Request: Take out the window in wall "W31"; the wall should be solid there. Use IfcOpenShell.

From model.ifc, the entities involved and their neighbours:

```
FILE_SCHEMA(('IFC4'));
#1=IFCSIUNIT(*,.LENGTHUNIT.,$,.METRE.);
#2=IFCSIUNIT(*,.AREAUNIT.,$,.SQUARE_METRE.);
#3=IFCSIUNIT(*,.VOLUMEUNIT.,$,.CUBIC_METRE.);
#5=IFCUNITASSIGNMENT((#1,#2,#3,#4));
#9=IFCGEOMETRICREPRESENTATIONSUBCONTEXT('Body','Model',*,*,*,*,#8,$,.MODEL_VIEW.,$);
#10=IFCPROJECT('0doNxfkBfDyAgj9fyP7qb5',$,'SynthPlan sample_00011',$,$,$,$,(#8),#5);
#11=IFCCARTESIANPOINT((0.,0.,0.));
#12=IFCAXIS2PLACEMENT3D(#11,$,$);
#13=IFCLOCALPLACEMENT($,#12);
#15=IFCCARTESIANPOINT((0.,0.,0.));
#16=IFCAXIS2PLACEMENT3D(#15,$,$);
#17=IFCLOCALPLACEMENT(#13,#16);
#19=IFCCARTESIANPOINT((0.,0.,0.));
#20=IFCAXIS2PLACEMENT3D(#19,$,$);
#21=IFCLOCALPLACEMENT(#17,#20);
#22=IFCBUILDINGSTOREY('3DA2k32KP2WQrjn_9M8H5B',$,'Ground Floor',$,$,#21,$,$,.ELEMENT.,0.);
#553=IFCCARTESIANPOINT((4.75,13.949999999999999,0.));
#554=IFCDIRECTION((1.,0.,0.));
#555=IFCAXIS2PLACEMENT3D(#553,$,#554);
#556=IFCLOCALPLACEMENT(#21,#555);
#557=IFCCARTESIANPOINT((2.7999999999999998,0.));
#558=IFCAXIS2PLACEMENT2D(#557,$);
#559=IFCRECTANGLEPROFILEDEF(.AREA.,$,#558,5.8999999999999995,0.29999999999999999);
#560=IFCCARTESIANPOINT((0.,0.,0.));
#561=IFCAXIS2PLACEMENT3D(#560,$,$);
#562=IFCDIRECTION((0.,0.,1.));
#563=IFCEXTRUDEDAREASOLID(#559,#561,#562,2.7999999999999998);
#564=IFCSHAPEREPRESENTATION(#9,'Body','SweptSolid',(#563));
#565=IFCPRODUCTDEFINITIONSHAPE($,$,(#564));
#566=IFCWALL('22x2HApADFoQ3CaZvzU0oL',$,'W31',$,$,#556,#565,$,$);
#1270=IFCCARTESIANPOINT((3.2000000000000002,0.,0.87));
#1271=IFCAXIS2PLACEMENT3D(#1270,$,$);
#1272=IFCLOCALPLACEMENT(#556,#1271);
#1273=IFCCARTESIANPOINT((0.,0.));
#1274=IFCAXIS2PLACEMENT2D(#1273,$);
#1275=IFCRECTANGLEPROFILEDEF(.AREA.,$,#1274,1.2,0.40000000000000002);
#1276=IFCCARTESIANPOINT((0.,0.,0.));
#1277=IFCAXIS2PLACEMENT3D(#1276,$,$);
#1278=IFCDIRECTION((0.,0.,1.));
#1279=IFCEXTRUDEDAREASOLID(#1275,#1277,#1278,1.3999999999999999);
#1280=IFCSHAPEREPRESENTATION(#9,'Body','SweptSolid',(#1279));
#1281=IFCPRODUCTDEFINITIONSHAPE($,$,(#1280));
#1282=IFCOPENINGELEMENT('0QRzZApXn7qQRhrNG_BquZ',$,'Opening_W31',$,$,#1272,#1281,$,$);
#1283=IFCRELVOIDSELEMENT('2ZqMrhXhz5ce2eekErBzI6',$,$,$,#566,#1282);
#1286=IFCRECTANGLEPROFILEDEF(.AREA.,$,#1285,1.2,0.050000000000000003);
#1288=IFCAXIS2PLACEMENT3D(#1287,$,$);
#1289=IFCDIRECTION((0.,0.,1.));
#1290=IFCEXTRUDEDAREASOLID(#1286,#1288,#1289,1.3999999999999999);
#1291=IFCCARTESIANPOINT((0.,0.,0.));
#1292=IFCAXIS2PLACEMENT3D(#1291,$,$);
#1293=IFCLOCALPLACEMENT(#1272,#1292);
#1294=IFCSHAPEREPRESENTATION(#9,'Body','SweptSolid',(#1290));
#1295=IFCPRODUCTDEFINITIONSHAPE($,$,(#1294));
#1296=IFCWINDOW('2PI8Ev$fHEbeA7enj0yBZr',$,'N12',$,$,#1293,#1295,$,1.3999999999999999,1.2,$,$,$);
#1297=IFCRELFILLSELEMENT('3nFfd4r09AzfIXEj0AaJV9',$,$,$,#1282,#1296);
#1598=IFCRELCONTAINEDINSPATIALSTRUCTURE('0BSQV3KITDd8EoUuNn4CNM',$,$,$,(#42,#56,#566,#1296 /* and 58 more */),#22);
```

```python
import ifcopenshell
import ifcopenshell.api.feature
import ifcopenshell.api.root
import ifcopenshell.geom
import ifcopenshell.util.shape

model = ifcopenshell.open("model.ifc")
settings = ifcopenshell.geom.settings()


def volume(element):
    """Net volume in cubic metres, openings subtracted."""
    shape = ifcopenshell.geom.create_shape(settings, element)
    return ifcopenshell.util.shape.get_volume(shape.geometry)


window = model.by_guid("2PI8Ev$fHEbeA7enj0yBZr")
opening = window.FillsVoids[0].RelatingOpeningElement
wall = opening.VoidsElements[0].RelatingBuildingElement
before = volume(wall)

ifcopenshell.api.root.remove_product(model, product=window)
ifcopenshell.api.feature.remove_feature(model, feature=opening)

after = volume(wall)

print(f"wall volume {before:.3f} -> {after:.3f} m3")

model.write("model_rev.ifc")
```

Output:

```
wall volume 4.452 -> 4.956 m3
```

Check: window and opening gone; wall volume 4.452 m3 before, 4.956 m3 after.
